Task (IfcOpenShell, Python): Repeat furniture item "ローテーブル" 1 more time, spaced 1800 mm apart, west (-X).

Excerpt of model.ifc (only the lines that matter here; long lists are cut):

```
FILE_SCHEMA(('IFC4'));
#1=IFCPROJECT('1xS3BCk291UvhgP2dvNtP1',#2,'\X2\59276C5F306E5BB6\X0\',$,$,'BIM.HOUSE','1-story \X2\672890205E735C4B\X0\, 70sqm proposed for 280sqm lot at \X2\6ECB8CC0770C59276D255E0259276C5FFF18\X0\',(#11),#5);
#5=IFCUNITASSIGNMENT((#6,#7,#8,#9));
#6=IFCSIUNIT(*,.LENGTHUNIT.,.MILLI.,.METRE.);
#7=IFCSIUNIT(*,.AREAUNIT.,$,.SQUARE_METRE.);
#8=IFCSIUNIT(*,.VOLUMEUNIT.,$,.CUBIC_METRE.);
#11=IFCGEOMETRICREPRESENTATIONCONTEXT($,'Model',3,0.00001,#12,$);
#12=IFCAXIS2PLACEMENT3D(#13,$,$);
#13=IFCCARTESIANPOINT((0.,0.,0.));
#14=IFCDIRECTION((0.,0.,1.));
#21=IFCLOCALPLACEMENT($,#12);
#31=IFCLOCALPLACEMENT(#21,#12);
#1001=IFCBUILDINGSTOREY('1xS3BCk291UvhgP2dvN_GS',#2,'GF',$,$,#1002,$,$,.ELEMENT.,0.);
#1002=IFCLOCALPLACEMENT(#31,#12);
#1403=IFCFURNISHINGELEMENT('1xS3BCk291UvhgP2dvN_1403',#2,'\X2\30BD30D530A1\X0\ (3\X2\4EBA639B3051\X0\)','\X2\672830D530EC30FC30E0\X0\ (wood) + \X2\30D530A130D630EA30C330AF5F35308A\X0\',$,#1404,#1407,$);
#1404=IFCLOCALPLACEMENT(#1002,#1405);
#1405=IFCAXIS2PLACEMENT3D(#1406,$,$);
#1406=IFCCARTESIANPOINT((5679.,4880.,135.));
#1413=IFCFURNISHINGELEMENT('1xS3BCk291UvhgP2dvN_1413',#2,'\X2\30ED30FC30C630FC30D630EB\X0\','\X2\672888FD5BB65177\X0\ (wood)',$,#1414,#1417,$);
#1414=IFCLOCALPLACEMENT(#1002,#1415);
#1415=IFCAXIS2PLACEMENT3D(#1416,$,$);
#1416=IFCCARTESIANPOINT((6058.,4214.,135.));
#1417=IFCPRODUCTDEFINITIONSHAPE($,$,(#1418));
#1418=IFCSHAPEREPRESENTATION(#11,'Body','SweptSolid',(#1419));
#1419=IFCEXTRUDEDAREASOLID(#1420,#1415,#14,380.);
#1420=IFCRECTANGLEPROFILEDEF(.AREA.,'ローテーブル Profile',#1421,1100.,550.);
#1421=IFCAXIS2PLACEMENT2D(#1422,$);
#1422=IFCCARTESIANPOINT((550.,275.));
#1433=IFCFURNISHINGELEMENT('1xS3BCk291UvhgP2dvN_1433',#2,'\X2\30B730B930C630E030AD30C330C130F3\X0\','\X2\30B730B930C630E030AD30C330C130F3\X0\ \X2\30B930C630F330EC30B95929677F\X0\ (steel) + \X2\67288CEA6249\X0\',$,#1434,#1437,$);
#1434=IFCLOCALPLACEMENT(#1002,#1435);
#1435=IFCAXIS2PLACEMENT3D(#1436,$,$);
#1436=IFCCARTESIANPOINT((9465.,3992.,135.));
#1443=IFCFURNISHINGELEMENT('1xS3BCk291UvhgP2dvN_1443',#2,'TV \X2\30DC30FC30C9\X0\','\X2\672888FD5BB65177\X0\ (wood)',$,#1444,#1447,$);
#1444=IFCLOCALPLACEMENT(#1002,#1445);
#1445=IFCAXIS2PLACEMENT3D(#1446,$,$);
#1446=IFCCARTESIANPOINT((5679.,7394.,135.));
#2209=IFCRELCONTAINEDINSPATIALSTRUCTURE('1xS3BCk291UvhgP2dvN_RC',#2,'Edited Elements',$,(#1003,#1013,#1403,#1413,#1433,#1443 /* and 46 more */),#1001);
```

```python
import numpy as np
import ifcopenshell
import ifcopenshell.api.geometry
import ifcopenshell.api.root
import ifcopenshell.util.element
import ifcopenshell.util.placement

model = ifcopenshell.open("model.ifc")


def reuse_history(source, copy):
    """copy_class also copies each property set's owner history, people and application; keep the originals."""
    for rel in copy.IsDefinedBy:
        if rel.is_a("IfcRelDefinesByProperties") and (history := rel.RelatingPropertyDefinition.OwnerHistory):
            rel.RelatingPropertyDefinition.OwnerHistory = source.OwnerHistory
            ifcopenshell.util.element.remove_deep2(model, history)


source = model.by_id(1413)
base = ifcopenshell.util.placement.get_local_placement(source.ObjectPlacement)
step = np.array([-1.0, 0.0, 0.0]) * 1800.0

for i in range(1, 2):
    copy = ifcopenshell.api.root.copy_class(model, product=source)
    copy.Representation = ifcopenshell.util.element.copy_deep(
        model, source.Representation, exclude=["IfcGeometricRepresentationContext", "IfcRepresentationMap"]
    )
    reuse_history(source, copy)
    matrix = base.copy()
    matrix[:3, 3] += i * step
    print("added at", matrix[:3, 3].round(3) + 0.0)
    ifcopenshell.api.geometry.edit_object_placement(model, product=copy, matrix=matrix, is_si=False)

model.write("model_rev.ifc")
```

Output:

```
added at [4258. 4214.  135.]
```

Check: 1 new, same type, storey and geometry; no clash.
